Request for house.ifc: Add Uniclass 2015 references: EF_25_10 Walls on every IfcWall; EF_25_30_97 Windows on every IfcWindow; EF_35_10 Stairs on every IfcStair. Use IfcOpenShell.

First a look at what the model holds.

```python
import ifcopenshell

model = ifcopenshell.open("house.ifc")
print(model.schema)
print("classifications:", [c.Name for c in model.by_type("IfcClassification")])
for ifc_class in ("IfcDoor", "IfcRoof", "IfcStair", "IfcWall", "IfcWindow"):
    print(ifc_class, len(model.by_type(ifc_class)))
```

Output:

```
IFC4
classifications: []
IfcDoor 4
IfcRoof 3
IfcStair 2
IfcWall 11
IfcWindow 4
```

```python
import ifcopenshell
import ifcopenshell.api.classification

model = ifcopenshell.open("house.ifc")

system = ifcopenshell.api.classification.add_classification(model, classification="Uniclass 2015")

codes = {
    "IfcWall": ("EF_25_10", "Walls"),
    "IfcWindow": ("EF_25_30_97", "Windows"),
    "IfcStair": ("EF_35_10", "Stairs"),
}
for ifc_class, (code, name) in codes.items():
    products = model.by_type(ifc_class)
    ifcopenshell.api.classification.add_reference(
        model, products=products, classification=system, identification=code, name=name
    )
    print(code, len(products))

model.write("house_updated.ifc")
```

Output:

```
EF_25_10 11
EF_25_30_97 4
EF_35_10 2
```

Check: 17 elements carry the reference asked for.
